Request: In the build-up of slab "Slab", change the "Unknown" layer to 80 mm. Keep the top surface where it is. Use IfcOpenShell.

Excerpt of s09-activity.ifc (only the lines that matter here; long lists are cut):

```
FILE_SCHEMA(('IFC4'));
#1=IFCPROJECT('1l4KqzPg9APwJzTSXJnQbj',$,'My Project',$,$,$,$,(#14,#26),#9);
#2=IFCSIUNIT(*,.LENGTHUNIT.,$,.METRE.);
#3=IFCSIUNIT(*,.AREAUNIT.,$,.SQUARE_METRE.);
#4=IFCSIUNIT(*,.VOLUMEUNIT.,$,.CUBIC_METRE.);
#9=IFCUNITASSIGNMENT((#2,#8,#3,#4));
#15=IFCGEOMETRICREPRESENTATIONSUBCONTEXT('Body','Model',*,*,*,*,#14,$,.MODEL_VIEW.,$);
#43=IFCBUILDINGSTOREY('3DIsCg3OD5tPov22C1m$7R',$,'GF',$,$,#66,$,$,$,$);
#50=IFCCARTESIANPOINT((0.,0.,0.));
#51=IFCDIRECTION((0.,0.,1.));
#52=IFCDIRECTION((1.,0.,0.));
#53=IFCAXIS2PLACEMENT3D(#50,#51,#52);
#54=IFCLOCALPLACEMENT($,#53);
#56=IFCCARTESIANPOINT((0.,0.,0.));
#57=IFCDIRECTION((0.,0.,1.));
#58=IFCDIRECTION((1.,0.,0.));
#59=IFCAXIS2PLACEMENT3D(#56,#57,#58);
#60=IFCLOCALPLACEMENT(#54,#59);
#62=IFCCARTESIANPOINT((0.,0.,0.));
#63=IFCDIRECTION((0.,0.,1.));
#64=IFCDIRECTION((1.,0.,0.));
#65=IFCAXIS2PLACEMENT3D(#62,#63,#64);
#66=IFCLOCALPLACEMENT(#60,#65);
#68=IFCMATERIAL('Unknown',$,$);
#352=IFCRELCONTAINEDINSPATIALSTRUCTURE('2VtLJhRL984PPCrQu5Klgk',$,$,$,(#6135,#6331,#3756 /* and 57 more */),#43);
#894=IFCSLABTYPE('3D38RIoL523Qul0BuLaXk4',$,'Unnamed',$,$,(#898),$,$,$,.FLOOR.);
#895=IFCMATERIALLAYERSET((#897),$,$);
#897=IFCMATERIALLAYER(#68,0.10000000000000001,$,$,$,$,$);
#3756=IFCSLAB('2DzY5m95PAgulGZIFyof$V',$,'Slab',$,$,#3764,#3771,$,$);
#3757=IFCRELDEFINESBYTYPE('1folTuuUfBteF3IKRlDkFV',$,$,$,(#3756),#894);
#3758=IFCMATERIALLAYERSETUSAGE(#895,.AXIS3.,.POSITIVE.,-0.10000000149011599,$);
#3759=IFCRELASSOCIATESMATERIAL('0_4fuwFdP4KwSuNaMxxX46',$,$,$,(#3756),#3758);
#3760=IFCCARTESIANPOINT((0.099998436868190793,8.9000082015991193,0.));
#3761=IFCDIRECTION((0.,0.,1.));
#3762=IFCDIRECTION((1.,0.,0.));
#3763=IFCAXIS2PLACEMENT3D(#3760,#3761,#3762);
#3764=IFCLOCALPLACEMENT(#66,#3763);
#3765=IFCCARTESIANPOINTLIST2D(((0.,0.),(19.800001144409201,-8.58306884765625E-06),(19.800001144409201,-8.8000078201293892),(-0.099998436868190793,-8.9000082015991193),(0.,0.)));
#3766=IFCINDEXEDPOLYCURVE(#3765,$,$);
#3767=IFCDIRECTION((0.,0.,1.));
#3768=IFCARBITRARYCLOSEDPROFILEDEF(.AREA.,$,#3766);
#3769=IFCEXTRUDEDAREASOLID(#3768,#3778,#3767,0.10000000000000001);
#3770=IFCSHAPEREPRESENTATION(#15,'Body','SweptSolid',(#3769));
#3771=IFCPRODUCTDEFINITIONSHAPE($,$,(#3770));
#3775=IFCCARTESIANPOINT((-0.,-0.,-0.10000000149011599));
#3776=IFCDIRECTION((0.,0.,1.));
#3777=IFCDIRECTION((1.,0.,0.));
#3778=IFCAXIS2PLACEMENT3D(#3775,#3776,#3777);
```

```python
import ifcopenshell
import ifcopenshell.util.element
import ifcopenshell.util.representation

model = ifcopenshell.open("s09-activity.ifc")

layer_set = model.by_id(895)
layer = next(l for l in layer_set.MaterialLayers if l.Material and l.Material.Name == "Unknown")
change = 0.08 - layer.LayerThickness
layer.LayerThickness += change

# Geometry does not follow the layer set by itself.
slabs = [e for e in ifcopenshell.util.element.get_elements_by_material(model, layer_set) if e.is_a("IfcSlab")]
for slab in sorted(slabs, key=lambda e: e.id()):
    body = ifcopenshell.util.representation.get_representation(slab, "Model", "Body")
    solid = body.Items[0]
    old_depth = solid.Depth
    solid.Depth += change
    # Extruded upwards: lower the start of the extrusion so the top stays.
    x, y, z = solid.Position.Location.Coordinates
    solid.Position.Location = model.createIfcCartesianPoint((x, y, z - change))
    print(slab.id(), f"{old_depth:g} -> {solid.Depth:g}")

# The layers are counted up from the underside, which has moved.
for usage in {ifcopenshell.util.element.get_material(slab) for slab in slabs}:
    usage.OffsetFromReferenceLine -= change

model.write("s09-activity_rev.ifc")
```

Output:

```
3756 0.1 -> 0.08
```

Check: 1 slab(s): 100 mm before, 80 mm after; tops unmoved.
